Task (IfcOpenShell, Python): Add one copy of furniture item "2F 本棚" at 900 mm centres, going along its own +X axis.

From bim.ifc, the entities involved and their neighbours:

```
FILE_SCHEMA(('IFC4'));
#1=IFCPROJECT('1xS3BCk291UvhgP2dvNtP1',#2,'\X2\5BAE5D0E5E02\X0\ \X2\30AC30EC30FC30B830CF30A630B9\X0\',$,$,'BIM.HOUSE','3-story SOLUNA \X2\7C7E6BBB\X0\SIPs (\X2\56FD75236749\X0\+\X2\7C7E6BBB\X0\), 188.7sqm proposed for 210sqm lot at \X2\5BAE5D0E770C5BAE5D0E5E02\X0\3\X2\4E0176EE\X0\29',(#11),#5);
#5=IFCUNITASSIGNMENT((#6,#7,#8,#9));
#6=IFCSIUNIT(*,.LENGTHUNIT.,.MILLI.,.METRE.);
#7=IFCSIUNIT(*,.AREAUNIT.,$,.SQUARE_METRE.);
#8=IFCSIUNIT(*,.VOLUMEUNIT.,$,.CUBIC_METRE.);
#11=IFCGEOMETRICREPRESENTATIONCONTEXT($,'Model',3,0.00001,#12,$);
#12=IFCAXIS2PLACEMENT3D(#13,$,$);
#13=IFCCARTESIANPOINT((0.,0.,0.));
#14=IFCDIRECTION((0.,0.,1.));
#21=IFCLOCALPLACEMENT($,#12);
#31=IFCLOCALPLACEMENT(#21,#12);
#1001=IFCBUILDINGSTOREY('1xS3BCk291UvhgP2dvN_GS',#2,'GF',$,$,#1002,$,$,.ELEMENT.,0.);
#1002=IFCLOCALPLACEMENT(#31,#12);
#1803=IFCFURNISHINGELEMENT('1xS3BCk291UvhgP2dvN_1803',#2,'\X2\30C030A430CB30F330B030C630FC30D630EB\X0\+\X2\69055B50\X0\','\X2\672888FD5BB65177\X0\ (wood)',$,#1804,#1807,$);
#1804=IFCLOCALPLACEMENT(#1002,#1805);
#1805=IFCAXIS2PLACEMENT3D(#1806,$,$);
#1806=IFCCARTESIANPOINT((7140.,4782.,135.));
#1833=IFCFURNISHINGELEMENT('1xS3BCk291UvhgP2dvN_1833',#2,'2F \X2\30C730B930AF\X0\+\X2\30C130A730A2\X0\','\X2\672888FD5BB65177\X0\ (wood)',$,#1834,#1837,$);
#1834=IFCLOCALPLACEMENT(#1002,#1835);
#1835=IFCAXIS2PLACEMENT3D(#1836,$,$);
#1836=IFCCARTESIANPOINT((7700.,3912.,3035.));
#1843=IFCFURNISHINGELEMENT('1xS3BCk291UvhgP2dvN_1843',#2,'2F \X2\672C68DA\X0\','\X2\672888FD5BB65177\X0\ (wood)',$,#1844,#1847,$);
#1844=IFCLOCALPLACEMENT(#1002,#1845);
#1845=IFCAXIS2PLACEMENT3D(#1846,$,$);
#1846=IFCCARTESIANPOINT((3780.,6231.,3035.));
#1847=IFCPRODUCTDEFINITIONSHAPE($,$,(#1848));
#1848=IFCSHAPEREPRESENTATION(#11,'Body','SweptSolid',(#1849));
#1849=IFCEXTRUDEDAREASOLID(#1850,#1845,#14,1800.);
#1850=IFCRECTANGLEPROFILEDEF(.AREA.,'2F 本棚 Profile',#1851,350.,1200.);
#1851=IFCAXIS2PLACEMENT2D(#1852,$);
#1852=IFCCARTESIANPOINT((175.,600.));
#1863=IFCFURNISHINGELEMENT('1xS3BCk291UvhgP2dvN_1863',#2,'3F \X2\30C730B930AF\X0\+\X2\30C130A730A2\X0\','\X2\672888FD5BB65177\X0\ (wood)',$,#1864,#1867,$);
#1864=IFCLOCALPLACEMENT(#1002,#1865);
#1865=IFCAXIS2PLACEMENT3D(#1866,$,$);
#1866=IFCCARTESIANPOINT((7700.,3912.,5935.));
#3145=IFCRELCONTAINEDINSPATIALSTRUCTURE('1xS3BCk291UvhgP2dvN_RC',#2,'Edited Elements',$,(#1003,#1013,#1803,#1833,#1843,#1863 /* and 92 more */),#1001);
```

```python
import ifcopenshell
import ifcopenshell.api.geometry
import ifcopenshell.api.root
import ifcopenshell.util.element
import ifcopenshell.util.placement
import ifcopenshell.util.unit

model = ifcopenshell.open("bim.ifc")
unit_scale = ifcopenshell.util.unit.calculate_unit_scale(model)


def reuse_history(source, copy):
    """copy_class also copies each property set's owner history, people and application; keep the originals."""
    for rel in copy.IsDefinedBy:
        if rel.is_a("IfcRelDefinesByProperties") and (history := rel.RelatingPropertyDefinition.OwnerHistory):
            rel.RelatingPropertyDefinition.OwnerHistory = source.OwnerHistory
            ifcopenshell.util.element.remove_deep2(model, history)


source = model.by_id(1843)
base = ifcopenshell.util.placement.get_local_placement(source.ObjectPlacement)
step = base[:3, 0] * 0.9 / unit_scale

for i in range(1, 2):
    copy = ifcopenshell.api.root.copy_class(model, product=source)
    copy.Representation = ifcopenshell.util.element.copy_deep(
        model, source.Representation, exclude=["IfcGeometricRepresentationContext", "IfcRepresentationMap"]
    )
    reuse_history(source, copy)
    matrix = base.copy()
    matrix[:3, 3] += i * step
    print("added at", matrix[:3, 3].round(3) + 0.0)
    ifcopenshell.api.geometry.edit_object_placement(model, product=copy, matrix=matrix, is_si=False)

model.write("bim_edited.ifc")
```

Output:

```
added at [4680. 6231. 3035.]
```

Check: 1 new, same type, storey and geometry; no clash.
